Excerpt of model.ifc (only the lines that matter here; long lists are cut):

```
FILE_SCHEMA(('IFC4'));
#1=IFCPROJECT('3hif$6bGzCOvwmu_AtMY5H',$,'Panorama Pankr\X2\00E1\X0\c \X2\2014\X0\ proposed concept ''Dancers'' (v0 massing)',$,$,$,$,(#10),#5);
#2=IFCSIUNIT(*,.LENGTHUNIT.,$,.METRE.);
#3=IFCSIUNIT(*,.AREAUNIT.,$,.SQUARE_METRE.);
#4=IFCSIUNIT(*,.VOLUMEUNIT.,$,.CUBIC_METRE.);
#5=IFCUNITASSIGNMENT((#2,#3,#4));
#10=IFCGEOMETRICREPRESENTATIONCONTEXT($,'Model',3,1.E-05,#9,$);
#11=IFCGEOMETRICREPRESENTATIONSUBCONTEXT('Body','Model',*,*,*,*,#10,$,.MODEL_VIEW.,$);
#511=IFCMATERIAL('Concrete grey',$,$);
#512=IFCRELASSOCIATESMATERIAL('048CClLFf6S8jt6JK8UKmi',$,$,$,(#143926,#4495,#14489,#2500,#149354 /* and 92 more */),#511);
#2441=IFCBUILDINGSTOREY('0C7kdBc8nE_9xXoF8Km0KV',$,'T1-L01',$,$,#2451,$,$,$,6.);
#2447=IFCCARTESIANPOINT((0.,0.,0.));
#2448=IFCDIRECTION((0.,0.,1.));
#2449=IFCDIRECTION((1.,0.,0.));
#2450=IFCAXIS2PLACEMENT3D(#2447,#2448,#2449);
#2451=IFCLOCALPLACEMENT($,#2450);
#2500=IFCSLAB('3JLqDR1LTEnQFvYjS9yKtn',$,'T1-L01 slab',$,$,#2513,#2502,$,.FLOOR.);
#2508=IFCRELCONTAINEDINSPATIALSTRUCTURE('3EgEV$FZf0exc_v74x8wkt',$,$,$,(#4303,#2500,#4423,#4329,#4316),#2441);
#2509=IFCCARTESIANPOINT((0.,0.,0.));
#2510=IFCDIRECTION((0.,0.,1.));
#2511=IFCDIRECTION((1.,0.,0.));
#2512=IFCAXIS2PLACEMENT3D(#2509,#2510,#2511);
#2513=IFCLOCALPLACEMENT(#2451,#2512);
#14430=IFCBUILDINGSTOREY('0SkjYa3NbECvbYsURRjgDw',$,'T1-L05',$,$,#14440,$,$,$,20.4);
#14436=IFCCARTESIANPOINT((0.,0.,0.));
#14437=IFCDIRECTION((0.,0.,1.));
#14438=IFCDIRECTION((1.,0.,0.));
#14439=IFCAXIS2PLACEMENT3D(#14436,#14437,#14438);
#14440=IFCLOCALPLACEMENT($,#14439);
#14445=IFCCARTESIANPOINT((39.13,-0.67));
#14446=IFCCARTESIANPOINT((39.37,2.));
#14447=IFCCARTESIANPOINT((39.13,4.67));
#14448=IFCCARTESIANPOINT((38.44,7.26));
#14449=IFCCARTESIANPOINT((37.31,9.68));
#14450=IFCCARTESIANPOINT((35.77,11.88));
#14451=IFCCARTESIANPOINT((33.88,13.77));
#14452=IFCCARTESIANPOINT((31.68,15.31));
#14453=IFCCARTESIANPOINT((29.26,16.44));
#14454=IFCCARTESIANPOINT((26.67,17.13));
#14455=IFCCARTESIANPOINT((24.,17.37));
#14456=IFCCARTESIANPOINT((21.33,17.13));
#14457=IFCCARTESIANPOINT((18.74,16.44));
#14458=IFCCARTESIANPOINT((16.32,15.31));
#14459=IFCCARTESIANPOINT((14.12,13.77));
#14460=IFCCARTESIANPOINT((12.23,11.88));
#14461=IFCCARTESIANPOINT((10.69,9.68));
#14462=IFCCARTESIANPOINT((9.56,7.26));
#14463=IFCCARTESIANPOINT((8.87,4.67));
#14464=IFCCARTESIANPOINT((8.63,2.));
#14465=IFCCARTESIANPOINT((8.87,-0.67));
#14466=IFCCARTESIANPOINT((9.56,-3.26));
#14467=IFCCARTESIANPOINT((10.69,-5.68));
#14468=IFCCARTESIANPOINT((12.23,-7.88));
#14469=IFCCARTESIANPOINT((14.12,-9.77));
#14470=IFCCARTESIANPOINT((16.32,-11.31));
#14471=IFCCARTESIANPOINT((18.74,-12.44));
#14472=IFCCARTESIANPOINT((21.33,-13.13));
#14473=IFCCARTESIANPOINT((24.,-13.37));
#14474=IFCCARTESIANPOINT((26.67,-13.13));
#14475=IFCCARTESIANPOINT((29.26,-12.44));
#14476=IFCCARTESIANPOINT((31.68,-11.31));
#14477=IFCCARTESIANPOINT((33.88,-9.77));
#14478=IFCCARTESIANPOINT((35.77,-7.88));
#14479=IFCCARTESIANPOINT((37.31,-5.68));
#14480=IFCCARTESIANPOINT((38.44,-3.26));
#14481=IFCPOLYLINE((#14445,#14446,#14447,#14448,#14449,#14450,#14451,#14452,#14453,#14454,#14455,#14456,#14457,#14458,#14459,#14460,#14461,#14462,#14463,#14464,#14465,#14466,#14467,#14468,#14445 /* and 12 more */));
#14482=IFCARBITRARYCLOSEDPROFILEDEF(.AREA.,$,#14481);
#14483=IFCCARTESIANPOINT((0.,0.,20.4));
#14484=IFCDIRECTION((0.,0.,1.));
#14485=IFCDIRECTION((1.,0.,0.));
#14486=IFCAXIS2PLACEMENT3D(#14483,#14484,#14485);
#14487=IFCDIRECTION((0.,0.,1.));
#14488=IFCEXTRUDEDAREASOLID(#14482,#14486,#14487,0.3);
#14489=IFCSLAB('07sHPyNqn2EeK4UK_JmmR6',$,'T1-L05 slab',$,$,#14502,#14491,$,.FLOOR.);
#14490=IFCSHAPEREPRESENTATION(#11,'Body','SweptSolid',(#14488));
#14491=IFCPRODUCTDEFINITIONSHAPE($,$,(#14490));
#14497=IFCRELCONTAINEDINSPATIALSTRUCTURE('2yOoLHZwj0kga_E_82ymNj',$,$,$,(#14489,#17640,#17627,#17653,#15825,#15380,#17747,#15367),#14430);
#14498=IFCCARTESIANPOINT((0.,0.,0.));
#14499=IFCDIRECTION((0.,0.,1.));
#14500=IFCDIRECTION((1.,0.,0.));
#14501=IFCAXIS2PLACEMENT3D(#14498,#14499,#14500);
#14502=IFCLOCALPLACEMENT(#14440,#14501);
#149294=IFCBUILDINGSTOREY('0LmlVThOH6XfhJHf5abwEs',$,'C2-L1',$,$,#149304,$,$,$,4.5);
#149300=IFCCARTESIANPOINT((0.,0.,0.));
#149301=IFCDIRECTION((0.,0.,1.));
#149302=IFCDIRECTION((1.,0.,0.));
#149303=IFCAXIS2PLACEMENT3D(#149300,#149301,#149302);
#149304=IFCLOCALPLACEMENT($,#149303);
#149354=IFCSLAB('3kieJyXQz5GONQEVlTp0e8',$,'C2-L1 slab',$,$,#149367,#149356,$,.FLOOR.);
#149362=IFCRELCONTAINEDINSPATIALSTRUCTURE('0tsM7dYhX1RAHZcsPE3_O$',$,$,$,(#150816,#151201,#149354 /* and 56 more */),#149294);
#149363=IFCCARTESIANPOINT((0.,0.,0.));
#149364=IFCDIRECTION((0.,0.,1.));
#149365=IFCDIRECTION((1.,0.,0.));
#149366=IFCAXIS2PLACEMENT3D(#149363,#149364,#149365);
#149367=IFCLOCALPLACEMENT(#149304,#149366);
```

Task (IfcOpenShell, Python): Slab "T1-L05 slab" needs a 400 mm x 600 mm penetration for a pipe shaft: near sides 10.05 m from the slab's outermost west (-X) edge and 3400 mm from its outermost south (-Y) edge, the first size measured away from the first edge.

```python
import numpy as np
import ifcopenshell
import ifcopenshell.api.feature
import ifcopenshell.api.geometry
import ifcopenshell.api.root
import ifcopenshell.geom
import ifcopenshell.util.placement
import ifcopenshell.util.representation
import ifcopenshell.util.shape
import ifcopenshell.util.unit

model = ifcopenshell.open("model.ifc")
unit_scale = ifcopenshell.util.unit.calculate_unit_scale(model)
settings = ifcopenshell.geom.settings()


def volume(element):
    """Net volume in cubic metres, openings subtracted."""
    shape = ifcopenshell.geom.create_shape(settings, element)
    return ifcopenshell.util.shape.get_volume(shape.geometry)


slab = model.by_guid("07sHPyNqn2EeK4UK_JmmR6")
before = volume(slab)

# Extent in the slab's own axes, in metres. The edges named are its -X and -Y sides.
slab_shape = ifcopenshell.geom.create_shape(settings, slab)
vertices = ifcopenshell.util.shape.get_vertices(slab_shape.geometry)
x_min, y_min, bottom = vertices.min(axis=0)
top = vertices[:, 2].max()

opening = ifcopenshell.api.root.create_entity(model, ifc_class="IfcOpeningElement", name="Pipe shaft opening", predefined_type="OPENING")
context = ifcopenshell.util.representation.get_context(model, "Model", "Body", "MODEL_VIEW")
width, depth = 0.4, 0.6
outline = [(0.0, 0.0), (width, 0.0), (width, depth), (0.0, depth), (0.0, 0.0)]
# Overshoot both faces by 50 mm so the cut is clean.
shape = ifcopenshell.api.geometry.add_slab_representation(
    model, context=context, depth=top - bottom + 0.1, polyline=outline
)
ifcopenshell.api.geometry.assign_representation(model, product=opening, representation=shape)

matrix = ifcopenshell.util.placement.get_local_placement(slab.ObjectPlacement)
matrix[:, 3] = matrix @ np.append(np.array([x_min + 10.05, y_min + 3.4, bottom - 0.05]) / unit_scale, 1.0)
ifcopenshell.api.geometry.edit_object_placement(model, product=opening, matrix=matrix, is_si=False)
ifcopenshell.api.feature.add_feature(model, feature=opening, element=slab)

after = volume(slab)

print(f"slab volume {before:.3f} -> {after:.3f} m3")

model.write("model_edited.ifc")
```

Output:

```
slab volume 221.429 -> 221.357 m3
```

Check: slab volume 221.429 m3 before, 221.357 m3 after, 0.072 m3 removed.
